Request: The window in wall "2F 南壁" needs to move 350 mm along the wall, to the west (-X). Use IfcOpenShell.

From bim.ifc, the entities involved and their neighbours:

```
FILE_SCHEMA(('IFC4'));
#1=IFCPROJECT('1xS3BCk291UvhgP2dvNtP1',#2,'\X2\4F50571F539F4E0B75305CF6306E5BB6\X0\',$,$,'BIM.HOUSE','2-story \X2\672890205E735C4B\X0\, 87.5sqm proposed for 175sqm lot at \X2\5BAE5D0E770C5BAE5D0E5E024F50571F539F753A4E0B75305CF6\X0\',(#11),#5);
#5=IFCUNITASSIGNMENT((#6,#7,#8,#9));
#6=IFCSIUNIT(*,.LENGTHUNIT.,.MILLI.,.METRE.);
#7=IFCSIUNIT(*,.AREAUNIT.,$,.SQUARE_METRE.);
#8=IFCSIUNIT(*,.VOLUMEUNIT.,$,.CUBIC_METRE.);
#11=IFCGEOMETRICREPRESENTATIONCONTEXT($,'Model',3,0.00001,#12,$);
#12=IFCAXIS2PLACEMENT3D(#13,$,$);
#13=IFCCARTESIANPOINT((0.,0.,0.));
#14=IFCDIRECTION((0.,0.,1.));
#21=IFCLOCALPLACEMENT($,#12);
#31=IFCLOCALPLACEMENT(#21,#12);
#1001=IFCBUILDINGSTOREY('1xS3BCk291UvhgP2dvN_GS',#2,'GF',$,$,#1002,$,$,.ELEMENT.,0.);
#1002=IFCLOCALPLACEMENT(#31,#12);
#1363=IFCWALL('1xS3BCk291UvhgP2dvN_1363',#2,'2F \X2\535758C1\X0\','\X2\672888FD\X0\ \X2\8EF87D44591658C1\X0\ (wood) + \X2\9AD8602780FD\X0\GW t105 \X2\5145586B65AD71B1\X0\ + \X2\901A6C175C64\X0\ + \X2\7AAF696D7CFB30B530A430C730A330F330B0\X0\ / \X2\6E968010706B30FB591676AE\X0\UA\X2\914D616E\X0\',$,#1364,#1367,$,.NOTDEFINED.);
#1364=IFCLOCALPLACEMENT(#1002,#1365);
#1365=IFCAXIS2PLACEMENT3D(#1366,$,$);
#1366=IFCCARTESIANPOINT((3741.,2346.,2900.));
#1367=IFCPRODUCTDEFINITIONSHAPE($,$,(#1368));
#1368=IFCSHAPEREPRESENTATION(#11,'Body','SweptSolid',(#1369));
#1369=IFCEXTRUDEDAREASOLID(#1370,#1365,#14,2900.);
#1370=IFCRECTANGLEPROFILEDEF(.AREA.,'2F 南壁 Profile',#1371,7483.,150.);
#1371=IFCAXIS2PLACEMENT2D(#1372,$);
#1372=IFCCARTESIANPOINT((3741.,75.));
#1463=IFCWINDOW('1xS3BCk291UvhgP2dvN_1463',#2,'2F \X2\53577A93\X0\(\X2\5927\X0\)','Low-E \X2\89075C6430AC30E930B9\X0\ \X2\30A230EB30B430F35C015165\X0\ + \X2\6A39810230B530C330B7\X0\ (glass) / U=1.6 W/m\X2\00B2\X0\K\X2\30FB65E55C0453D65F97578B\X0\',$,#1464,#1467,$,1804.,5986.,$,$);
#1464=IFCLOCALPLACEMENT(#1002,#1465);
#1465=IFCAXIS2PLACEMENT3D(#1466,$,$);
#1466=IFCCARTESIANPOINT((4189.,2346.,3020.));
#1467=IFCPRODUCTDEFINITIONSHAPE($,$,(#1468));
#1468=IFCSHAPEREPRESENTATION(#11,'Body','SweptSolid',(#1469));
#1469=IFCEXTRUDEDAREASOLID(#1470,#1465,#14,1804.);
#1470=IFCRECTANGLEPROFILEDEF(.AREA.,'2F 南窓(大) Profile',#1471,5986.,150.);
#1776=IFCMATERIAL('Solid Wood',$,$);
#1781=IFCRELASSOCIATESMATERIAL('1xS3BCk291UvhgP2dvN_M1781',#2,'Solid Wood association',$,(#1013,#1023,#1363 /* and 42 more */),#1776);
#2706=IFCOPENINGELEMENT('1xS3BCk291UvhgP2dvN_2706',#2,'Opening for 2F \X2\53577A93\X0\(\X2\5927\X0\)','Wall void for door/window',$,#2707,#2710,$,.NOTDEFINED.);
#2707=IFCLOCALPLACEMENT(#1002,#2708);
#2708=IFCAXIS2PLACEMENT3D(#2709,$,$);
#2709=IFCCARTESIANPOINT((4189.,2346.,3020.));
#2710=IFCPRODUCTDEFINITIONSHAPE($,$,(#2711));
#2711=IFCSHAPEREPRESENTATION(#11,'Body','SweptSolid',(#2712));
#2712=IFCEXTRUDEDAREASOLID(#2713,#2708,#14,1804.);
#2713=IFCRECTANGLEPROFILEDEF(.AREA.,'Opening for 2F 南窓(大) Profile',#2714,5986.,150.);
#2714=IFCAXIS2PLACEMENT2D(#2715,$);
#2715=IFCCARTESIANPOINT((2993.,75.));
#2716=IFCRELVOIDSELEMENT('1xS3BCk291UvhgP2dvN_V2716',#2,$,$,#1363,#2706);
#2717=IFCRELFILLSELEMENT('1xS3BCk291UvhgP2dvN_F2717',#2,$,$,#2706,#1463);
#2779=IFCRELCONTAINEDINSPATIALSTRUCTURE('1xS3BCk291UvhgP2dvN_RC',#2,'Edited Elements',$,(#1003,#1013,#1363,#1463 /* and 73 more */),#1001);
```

```python
import ifcopenshell
import ifcopenshell.api.geometry
import ifcopenshell.util.placement
import ifcopenshell.util.unit

model = ifcopenshell.open("bim.ifc")
unit_scale = ifcopenshell.util.unit.calculate_unit_scale(model)

window = model.by_guid("1xS3BCk291UvhgP2dvN_1463")
opening = window.FillsVoids[0].RelatingOpeningElement
wall = opening.VoidsElements[0].RelatingBuildingElement

wall_matrix = ifcopenshell.util.placement.get_local_placement(wall.ObjectPlacement)
shift = wall_matrix[:3, 0] * -0.35 / unit_scale
before = ifcopenshell.util.placement.get_local_placement(window.ObjectPlacement)[:3, 3].copy()

# The window is not placed relative to its opening, so move both.
for product in (opening, window):
    matrix = ifcopenshell.util.placement.get_local_placement(product.ObjectPlacement)
    matrix[:3, 3] += shift
    ifcopenshell.api.geometry.edit_object_placement(model, product=product, matrix=matrix, is_si=False)

after = ifcopenshell.util.placement.get_local_placement(window.ObjectPlacement)[:3, 3]
print("window moved by", (after - before).round(3) + 0.0)

model.write("bim_rev.ifc")
```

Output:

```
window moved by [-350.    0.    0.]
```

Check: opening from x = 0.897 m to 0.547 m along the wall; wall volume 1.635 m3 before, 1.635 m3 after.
